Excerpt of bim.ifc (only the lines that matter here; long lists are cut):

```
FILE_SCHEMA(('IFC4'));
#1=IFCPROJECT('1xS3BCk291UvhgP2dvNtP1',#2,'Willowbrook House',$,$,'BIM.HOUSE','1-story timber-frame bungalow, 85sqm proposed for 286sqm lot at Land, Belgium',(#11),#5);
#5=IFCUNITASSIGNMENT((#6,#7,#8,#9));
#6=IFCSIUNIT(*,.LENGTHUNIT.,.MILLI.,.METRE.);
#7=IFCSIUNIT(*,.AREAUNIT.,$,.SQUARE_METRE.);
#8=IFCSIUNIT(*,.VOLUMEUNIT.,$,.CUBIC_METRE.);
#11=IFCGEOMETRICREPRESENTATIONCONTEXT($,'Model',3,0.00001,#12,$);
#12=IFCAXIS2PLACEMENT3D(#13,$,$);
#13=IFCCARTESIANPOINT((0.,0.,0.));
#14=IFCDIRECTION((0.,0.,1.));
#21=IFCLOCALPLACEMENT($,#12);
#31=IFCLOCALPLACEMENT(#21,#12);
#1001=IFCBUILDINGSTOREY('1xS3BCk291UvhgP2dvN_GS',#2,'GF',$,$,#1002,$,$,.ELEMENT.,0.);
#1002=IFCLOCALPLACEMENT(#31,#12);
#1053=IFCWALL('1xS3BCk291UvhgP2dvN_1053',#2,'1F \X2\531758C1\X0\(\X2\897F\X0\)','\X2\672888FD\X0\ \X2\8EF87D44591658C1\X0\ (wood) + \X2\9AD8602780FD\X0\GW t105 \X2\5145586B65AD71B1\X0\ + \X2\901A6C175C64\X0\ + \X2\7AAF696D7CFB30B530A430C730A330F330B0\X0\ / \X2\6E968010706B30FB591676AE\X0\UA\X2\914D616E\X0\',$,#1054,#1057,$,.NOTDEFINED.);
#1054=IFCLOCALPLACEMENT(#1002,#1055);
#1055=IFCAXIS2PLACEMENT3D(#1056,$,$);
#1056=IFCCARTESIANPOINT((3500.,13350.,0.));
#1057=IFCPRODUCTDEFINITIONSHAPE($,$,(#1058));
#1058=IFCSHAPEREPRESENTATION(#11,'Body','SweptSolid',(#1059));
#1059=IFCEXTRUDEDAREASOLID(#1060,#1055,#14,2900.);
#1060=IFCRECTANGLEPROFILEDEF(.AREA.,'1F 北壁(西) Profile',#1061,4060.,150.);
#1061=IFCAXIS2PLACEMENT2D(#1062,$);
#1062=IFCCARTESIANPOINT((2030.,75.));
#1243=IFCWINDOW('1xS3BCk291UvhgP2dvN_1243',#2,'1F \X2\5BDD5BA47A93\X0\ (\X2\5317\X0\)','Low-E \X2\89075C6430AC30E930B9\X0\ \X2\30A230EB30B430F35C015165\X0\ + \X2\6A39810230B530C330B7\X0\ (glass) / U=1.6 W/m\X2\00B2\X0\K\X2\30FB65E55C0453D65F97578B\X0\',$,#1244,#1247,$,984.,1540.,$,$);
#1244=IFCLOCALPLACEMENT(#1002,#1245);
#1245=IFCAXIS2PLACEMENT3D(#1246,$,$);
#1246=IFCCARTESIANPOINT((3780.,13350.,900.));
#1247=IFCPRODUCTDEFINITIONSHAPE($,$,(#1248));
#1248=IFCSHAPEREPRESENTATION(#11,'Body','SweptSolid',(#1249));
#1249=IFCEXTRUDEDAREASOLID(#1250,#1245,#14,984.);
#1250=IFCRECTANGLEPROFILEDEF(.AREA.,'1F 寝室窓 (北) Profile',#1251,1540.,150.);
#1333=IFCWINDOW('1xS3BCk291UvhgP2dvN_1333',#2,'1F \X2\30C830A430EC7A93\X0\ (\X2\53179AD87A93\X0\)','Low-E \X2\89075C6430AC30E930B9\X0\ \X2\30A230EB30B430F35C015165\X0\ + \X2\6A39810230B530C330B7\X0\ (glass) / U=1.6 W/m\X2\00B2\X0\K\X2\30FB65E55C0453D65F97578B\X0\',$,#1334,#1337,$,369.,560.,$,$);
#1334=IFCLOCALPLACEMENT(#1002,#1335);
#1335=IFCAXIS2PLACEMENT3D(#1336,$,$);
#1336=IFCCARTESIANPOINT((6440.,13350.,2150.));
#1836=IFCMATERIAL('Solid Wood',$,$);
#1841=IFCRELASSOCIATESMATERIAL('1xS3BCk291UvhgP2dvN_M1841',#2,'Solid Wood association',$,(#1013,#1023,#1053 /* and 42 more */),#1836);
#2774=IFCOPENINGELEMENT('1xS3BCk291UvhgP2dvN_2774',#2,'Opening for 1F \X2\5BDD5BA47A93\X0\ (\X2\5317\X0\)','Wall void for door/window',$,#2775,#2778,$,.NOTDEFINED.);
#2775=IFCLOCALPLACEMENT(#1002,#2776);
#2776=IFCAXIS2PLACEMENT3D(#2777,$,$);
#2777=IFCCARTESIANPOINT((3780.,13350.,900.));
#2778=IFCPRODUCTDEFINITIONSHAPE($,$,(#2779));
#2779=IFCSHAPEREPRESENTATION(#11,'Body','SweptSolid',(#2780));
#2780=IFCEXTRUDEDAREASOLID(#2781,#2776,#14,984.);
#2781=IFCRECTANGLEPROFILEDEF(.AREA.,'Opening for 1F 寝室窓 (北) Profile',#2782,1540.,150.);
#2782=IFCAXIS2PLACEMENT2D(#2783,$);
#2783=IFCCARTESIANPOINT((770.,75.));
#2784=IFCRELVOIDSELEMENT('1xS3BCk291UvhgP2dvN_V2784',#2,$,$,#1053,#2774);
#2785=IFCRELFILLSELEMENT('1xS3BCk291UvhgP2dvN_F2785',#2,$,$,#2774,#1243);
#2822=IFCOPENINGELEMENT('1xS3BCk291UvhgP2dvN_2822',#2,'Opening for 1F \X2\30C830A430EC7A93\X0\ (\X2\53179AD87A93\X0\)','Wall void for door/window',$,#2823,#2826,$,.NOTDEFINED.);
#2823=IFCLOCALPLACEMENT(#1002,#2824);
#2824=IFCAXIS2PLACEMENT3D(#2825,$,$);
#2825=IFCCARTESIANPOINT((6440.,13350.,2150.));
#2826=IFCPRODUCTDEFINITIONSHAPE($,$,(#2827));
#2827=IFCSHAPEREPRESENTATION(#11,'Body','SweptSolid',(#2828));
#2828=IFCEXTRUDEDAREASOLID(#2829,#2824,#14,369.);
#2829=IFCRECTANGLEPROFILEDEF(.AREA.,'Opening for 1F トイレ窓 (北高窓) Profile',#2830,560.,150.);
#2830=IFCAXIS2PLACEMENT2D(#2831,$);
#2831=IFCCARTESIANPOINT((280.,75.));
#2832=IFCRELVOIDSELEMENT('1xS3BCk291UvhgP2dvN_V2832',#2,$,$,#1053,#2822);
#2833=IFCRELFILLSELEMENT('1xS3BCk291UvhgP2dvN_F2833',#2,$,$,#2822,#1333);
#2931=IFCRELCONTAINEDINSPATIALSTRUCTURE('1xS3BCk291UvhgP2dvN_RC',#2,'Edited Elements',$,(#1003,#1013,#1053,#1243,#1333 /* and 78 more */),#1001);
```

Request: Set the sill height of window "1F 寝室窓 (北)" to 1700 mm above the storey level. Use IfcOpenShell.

```python
import numpy as np
import ifcopenshell
import ifcopenshell.api.geometry
import ifcopenshell.geom
import ifcopenshell.util.element
import ifcopenshell.util.placement
import ifcopenshell.util.shape
import ifcopenshell.util.unit

model = ifcopenshell.open("bim.ifc")
unit_scale = ifcopenshell.util.unit.calculate_unit_scale(model)

window = model.by_id(1243)
opening = window.FillsVoids[0].RelatingOpeningElement
storey = ifcopenshell.util.element.get_container(window, ifc_class="IfcBuildingStorey")
level = ifcopenshell.util.placement.get_local_placement(storey.ObjectPlacement)[2, 3]

# The opening's origin need not be at the sill, so measure its lowest point.
shape = ifcopenshell.geom.create_shape(ifcopenshell.geom.settings(), opening)
bottom = ifcopenshell.util.shape.get_shape_bottom_elevation(shape, shape.geometry) / unit_scale
dz = level + 1.7 / unit_scale - bottom

shift = np.array([0.0, 0.0, dz])
# The window is not placed relative to its opening, so move both.
for product in (opening, window):
    matrix = ifcopenshell.util.placement.get_local_placement(product.ObjectPlacement)
    matrix[:3, 3] += shift
    ifcopenshell.api.geometry.edit_object_placement(model, product=product, matrix=matrix, is_si=False)

print(f"moved by {dz * unit_scale:+.3f} m")

model.write("bim_edited.ifc")
```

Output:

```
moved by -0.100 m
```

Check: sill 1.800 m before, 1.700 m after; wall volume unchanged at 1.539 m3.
